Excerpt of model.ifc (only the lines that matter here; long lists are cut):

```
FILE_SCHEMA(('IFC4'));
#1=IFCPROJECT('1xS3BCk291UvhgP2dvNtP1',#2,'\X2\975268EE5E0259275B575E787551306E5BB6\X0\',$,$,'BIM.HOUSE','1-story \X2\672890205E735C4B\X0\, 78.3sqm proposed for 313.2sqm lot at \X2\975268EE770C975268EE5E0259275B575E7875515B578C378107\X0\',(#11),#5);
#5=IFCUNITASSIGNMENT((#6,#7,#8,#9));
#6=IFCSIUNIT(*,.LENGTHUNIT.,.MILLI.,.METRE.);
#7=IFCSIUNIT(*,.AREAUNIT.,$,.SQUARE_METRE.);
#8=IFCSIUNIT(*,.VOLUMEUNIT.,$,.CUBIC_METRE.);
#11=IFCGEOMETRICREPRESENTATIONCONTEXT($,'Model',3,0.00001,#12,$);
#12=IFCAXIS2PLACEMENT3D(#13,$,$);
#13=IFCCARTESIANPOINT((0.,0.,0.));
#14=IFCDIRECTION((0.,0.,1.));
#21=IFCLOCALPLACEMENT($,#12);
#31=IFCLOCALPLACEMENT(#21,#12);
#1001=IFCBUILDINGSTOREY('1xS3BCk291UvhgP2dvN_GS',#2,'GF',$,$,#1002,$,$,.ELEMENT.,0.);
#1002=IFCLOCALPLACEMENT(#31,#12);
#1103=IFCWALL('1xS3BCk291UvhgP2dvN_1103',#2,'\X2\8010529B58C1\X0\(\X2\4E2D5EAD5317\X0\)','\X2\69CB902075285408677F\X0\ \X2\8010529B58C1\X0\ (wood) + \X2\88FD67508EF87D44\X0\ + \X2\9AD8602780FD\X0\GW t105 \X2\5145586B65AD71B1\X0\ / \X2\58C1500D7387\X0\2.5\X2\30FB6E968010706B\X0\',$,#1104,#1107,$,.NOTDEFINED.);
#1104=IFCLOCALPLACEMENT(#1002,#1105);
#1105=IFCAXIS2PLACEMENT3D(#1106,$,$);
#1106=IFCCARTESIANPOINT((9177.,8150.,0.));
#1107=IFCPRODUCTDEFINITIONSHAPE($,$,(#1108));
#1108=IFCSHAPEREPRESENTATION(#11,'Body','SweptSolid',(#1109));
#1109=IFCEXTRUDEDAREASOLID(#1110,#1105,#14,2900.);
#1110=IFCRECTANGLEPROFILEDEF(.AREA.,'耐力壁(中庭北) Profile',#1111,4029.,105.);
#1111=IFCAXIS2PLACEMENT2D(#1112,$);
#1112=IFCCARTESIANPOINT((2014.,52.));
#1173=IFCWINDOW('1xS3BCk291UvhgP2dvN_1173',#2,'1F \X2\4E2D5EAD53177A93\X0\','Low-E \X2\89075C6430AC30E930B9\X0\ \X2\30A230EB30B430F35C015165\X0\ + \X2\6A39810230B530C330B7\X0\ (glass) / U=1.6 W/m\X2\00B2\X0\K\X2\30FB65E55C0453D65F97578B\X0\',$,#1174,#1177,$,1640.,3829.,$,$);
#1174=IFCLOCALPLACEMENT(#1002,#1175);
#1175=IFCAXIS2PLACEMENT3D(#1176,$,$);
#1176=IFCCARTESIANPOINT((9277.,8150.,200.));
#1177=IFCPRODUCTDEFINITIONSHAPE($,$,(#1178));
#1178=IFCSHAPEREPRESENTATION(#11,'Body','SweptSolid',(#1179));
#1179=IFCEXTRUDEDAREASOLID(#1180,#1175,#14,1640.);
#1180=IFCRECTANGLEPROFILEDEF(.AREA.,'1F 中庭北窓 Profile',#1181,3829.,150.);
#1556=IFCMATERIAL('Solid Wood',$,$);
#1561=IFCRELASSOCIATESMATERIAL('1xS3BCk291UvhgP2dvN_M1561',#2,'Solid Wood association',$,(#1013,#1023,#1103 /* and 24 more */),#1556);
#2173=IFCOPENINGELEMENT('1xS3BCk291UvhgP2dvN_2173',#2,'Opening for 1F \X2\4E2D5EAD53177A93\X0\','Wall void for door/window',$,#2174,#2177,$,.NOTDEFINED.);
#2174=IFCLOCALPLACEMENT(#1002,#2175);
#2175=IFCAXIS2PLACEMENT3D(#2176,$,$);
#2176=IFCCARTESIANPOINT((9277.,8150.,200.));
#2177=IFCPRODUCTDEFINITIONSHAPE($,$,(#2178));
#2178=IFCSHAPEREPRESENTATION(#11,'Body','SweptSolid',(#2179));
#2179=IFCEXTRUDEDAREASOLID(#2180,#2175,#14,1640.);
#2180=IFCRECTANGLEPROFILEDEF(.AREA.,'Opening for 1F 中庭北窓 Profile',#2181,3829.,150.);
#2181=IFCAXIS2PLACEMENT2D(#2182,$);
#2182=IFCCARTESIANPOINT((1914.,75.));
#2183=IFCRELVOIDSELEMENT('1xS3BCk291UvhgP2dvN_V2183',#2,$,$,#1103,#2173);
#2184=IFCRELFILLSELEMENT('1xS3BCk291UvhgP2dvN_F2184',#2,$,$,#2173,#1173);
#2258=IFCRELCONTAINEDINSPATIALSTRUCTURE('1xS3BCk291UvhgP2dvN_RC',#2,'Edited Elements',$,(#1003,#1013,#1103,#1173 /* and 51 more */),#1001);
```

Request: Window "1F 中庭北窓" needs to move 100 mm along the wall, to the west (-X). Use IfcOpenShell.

```python
import ifcopenshell
import ifcopenshell.api.geometry
import ifcopenshell.util.placement

model = ifcopenshell.open("model.ifc")

window = model.by_guid("1xS3BCk291UvhgP2dvN_1173")
opening = window.FillsVoids[0].RelatingOpeningElement
wall = opening.VoidsElements[0].RelatingBuildingElement

wall_matrix = ifcopenshell.util.placement.get_local_placement(wall.ObjectPlacement)
shift = wall_matrix[:3, 0] * -100.0
before = ifcopenshell.util.placement.get_local_placement(window.ObjectPlacement)[:3, 3].copy()

# The window is not placed relative to its opening, so move both.
for product in (opening, window):
    matrix = ifcopenshell.util.placement.get_local_placement(product.ObjectPlacement)
    matrix[:3, 3] += shift
    ifcopenshell.api.geometry.edit_object_placement(model, product=product, matrix=matrix, is_si=False)

after = ifcopenshell.util.placement.get_local_placement(window.ObjectPlacement)[:3, 3]
print("window moved by", (after - before).round(3) + 0.0)

model.write("model_rev.ifc")
```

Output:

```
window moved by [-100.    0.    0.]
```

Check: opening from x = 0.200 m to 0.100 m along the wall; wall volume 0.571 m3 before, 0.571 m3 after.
